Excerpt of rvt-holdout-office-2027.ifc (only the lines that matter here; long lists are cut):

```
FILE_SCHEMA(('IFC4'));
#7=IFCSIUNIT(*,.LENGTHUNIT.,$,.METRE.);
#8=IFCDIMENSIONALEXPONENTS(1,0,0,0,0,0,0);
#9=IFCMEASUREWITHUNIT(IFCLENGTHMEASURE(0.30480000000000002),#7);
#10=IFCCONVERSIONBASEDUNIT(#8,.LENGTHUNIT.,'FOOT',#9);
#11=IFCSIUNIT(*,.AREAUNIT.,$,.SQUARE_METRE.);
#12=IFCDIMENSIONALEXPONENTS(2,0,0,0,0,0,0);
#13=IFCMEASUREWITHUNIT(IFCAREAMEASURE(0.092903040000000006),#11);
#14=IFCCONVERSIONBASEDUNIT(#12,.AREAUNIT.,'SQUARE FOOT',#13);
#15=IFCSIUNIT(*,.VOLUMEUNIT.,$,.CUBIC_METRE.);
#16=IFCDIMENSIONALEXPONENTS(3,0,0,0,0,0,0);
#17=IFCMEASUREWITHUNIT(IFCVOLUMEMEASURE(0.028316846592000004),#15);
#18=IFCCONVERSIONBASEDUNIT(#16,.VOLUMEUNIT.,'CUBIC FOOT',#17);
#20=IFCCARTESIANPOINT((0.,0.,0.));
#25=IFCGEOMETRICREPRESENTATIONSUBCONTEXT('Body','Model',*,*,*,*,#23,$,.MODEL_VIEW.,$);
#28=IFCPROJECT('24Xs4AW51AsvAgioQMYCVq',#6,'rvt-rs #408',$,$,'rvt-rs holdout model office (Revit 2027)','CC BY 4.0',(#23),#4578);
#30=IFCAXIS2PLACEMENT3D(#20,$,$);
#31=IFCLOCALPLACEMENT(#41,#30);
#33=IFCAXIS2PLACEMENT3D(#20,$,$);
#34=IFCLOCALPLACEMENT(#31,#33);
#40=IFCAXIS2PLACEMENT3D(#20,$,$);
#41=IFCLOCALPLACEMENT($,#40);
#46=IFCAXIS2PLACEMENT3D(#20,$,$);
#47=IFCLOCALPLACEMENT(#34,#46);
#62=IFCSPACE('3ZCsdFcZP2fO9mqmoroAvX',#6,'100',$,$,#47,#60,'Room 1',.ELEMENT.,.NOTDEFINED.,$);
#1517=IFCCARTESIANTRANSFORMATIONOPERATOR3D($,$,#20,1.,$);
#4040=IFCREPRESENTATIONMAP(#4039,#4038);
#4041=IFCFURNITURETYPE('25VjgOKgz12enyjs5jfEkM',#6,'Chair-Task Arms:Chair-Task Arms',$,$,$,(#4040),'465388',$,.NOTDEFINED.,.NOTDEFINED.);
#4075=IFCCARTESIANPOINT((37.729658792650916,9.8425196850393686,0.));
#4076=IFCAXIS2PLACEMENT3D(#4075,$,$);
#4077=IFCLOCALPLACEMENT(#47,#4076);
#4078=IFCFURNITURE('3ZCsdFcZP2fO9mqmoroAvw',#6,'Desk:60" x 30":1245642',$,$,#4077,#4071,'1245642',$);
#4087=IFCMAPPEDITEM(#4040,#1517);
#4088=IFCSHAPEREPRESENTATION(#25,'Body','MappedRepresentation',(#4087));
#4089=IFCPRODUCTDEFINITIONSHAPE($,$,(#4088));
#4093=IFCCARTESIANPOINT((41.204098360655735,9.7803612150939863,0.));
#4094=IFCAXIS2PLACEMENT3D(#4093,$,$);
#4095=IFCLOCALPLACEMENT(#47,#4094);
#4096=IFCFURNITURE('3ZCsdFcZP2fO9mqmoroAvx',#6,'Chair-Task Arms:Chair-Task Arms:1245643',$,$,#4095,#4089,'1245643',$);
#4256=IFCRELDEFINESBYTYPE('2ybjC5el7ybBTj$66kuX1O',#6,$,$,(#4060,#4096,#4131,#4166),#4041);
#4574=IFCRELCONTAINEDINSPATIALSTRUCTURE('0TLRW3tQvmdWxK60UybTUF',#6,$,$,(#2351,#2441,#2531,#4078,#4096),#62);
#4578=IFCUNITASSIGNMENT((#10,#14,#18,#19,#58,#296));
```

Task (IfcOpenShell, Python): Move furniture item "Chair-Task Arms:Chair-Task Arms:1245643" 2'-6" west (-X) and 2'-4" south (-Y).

```python
import ifcopenshell
import ifcopenshell.api.geometry
import ifcopenshell.util.placement
import ifcopenshell.util.unit

model = ifcopenshell.open("rvt-holdout-office-2027.ifc")
unit_scale = ifcopenshell.util.unit.calculate_unit_scale(model)

item = model.by_guid("3ZCsdFcZP2fO9mqmoroAvx")
matrix = ifcopenshell.util.placement.get_local_placement(item.ObjectPlacement)
matrix[0, 3] -= 30 * 0.0254 / unit_scale
matrix[1, 3] -= 28 * 0.0254 / unit_scale
ifcopenshell.api.geometry.edit_object_placement(model, product=item, matrix=matrix, is_si=False)

print(ifcopenshell.util.placement.get_local_placement(item.ObjectPlacement).round(3) + 0.0)

model.write("rvt-holdout-office-2027_updated.ifc")
```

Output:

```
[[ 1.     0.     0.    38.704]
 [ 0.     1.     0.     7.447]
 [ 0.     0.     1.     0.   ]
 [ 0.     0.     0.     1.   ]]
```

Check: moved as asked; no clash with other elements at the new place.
